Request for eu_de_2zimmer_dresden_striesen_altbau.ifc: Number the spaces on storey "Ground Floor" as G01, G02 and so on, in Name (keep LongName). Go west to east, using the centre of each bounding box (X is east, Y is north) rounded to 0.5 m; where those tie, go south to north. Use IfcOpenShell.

First a look at what the model holds.

```python
import ifcopenshell
import ifcopenshell.util.element
import ifcopenshell.util.placement

model = ifcopenshell.open("eu_de_2zimmer_dresden_striesen_altbau.ifc")
print(model.schema)
storey = next(s for s in model.by_type("IfcBuildingStorey") if s.Name == "Ground Floor")
spaces = [e for e in ifcopenshell.util.element.get_decomposition(storey) if e.is_a("IfcSpace")]
for e in sorted(spaces, key=lambda e: e.id()):
    origin = ifcopenshell.util.placement.get_local_placement(e.ObjectPlacement)[:3, 3]
    print(e.id(), e.Name, e.LongName, origin.round(2) + 0.0, sep=" | ")
```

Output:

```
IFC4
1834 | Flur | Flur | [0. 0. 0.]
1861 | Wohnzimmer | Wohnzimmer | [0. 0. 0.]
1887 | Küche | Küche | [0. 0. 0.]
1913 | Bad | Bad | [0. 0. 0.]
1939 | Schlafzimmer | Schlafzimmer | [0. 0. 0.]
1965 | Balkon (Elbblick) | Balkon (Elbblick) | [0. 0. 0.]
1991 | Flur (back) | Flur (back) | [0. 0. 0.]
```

```python
import ifcopenshell
import ifcopenshell.geom
import ifcopenshell.util.element
import ifcopenshell.util.shape

model = ifcopenshell.open("eu_de_2zimmer_dresden_striesen_altbau.ifc")
settings = ifcopenshell.geom.settings()
settings.set("use-world-coords", True)


def centre(element):
    shape = ifcopenshell.geom.create_shape(settings, element)
    return ifcopenshell.util.shape.get_bbox_centroid(shape.geometry)


storey = next(s for s in model.by_type("IfcBuildingStorey") if s.Name == "Ground Floor")
spaces = [e for e in ifcopenshell.util.element.get_decomposition(storey) if e.is_a("IfcSpace")]

# Insertion points can sit at a corner or the storey origin, so sort by the geometry (in metres).
centres = {e: centre(e) for e in spaces}
spaces.sort(key=lambda e: (round(centres[e][0] / 0.5), centres[e][1]))

for i, e in enumerate(spaces, start=1):
    number = f"G{i:02d}"
    e.Name = number
    print(e.id(), number)

model.write("eu_de_2zimmer_dresden_striesen_altbau_rev.ifc")
```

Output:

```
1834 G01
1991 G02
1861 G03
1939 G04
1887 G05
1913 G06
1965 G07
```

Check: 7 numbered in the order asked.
